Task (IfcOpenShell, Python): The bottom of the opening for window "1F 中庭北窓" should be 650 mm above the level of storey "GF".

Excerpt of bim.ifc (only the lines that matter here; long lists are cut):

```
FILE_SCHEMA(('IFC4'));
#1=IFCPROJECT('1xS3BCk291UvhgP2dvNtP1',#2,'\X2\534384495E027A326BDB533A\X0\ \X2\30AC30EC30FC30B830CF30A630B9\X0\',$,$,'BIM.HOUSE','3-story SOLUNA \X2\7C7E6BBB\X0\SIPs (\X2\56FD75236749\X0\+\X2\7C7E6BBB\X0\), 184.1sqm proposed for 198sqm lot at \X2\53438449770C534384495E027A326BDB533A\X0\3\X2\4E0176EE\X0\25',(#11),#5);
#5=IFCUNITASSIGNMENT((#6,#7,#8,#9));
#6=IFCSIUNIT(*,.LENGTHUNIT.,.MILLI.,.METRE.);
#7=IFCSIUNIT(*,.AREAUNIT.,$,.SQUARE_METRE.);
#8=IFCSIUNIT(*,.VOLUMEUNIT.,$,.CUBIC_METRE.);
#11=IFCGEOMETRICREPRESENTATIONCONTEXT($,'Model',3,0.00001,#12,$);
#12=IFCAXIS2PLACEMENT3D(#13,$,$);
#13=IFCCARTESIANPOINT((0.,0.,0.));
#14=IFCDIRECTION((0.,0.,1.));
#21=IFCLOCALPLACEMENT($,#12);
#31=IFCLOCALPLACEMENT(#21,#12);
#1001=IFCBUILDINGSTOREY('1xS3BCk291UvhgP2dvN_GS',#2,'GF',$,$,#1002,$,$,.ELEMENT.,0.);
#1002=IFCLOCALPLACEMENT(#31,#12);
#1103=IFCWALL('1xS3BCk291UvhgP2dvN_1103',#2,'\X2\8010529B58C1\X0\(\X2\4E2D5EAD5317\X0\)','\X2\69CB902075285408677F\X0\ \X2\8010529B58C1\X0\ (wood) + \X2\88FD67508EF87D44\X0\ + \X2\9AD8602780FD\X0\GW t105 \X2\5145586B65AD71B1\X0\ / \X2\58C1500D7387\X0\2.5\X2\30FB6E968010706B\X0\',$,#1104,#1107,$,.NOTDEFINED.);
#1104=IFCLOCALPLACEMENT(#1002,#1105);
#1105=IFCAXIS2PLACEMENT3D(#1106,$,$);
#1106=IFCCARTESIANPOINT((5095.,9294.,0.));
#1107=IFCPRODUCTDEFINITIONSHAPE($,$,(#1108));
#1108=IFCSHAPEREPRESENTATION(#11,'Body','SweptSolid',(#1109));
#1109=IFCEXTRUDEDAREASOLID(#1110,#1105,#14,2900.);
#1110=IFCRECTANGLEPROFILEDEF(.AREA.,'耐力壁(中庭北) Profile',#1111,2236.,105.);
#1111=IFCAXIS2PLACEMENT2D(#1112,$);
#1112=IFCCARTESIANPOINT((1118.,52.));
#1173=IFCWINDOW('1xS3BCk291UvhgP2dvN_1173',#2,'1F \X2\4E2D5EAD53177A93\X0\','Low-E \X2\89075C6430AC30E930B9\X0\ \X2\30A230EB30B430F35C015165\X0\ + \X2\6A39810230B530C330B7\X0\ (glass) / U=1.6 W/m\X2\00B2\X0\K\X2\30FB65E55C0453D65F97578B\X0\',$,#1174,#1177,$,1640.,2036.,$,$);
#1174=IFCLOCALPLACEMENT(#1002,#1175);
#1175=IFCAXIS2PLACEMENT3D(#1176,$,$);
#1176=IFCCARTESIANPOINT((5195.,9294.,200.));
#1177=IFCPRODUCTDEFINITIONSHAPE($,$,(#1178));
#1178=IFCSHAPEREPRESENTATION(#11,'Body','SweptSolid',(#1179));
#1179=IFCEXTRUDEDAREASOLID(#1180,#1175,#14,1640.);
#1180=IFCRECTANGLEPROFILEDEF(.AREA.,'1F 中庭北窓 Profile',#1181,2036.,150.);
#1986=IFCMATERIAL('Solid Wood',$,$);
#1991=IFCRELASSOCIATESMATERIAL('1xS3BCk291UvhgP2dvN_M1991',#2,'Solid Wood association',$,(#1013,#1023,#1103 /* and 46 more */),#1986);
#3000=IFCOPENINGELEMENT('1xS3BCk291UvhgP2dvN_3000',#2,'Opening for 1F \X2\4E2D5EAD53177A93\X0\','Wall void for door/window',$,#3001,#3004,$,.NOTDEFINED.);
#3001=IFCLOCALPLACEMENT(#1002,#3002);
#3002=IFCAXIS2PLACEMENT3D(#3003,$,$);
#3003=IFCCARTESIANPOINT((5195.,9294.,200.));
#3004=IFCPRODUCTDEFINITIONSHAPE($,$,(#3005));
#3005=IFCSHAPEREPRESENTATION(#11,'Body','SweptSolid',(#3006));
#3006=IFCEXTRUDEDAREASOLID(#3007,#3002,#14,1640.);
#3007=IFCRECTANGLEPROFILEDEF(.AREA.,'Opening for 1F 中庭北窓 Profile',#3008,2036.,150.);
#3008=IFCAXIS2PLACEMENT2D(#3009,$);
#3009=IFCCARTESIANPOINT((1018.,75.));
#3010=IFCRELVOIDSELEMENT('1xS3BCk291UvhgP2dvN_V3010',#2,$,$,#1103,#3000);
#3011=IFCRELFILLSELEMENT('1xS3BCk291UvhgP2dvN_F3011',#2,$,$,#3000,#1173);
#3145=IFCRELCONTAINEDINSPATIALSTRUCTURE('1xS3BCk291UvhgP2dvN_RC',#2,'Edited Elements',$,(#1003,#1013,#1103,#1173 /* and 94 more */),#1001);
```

```python
import numpy as np
import ifcopenshell
import ifcopenshell.api.geometry
import ifcopenshell.geom
import ifcopenshell.util.element
import ifcopenshell.util.placement
import ifcopenshell.util.shape
import ifcopenshell.util.unit

model = ifcopenshell.open("bim.ifc")
unit_scale = ifcopenshell.util.unit.calculate_unit_scale(model)

window = model.by_guid("1xS3BCk291UvhgP2dvN_1173")
opening = window.FillsVoids[0].RelatingOpeningElement
storey = ifcopenshell.util.element.get_container(window, ifc_class="IfcBuildingStorey")
level = ifcopenshell.util.placement.get_local_placement(storey.ObjectPlacement)[2, 3]

# The opening's origin need not be at the sill, so measure its lowest point.
shape = ifcopenshell.geom.create_shape(ifcopenshell.geom.settings(), opening)
bottom = ifcopenshell.util.shape.get_shape_bottom_elevation(shape, shape.geometry) / unit_scale
dz = level + 650.0 - bottom

shift = np.array([0.0, 0.0, dz])
# The window is not placed relative to its opening, so move both.
for product in (opening, window):
    matrix = ifcopenshell.util.placement.get_local_placement(product.ObjectPlacement)
    matrix[:3, 3] += shift
    ifcopenshell.api.geometry.edit_object_placement(model, product=product, matrix=matrix, is_si=False)

print(f"moved by {dz * unit_scale:+.3f} m")

model.write("bim_v2.ifc")
```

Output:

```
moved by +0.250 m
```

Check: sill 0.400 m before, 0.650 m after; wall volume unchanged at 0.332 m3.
